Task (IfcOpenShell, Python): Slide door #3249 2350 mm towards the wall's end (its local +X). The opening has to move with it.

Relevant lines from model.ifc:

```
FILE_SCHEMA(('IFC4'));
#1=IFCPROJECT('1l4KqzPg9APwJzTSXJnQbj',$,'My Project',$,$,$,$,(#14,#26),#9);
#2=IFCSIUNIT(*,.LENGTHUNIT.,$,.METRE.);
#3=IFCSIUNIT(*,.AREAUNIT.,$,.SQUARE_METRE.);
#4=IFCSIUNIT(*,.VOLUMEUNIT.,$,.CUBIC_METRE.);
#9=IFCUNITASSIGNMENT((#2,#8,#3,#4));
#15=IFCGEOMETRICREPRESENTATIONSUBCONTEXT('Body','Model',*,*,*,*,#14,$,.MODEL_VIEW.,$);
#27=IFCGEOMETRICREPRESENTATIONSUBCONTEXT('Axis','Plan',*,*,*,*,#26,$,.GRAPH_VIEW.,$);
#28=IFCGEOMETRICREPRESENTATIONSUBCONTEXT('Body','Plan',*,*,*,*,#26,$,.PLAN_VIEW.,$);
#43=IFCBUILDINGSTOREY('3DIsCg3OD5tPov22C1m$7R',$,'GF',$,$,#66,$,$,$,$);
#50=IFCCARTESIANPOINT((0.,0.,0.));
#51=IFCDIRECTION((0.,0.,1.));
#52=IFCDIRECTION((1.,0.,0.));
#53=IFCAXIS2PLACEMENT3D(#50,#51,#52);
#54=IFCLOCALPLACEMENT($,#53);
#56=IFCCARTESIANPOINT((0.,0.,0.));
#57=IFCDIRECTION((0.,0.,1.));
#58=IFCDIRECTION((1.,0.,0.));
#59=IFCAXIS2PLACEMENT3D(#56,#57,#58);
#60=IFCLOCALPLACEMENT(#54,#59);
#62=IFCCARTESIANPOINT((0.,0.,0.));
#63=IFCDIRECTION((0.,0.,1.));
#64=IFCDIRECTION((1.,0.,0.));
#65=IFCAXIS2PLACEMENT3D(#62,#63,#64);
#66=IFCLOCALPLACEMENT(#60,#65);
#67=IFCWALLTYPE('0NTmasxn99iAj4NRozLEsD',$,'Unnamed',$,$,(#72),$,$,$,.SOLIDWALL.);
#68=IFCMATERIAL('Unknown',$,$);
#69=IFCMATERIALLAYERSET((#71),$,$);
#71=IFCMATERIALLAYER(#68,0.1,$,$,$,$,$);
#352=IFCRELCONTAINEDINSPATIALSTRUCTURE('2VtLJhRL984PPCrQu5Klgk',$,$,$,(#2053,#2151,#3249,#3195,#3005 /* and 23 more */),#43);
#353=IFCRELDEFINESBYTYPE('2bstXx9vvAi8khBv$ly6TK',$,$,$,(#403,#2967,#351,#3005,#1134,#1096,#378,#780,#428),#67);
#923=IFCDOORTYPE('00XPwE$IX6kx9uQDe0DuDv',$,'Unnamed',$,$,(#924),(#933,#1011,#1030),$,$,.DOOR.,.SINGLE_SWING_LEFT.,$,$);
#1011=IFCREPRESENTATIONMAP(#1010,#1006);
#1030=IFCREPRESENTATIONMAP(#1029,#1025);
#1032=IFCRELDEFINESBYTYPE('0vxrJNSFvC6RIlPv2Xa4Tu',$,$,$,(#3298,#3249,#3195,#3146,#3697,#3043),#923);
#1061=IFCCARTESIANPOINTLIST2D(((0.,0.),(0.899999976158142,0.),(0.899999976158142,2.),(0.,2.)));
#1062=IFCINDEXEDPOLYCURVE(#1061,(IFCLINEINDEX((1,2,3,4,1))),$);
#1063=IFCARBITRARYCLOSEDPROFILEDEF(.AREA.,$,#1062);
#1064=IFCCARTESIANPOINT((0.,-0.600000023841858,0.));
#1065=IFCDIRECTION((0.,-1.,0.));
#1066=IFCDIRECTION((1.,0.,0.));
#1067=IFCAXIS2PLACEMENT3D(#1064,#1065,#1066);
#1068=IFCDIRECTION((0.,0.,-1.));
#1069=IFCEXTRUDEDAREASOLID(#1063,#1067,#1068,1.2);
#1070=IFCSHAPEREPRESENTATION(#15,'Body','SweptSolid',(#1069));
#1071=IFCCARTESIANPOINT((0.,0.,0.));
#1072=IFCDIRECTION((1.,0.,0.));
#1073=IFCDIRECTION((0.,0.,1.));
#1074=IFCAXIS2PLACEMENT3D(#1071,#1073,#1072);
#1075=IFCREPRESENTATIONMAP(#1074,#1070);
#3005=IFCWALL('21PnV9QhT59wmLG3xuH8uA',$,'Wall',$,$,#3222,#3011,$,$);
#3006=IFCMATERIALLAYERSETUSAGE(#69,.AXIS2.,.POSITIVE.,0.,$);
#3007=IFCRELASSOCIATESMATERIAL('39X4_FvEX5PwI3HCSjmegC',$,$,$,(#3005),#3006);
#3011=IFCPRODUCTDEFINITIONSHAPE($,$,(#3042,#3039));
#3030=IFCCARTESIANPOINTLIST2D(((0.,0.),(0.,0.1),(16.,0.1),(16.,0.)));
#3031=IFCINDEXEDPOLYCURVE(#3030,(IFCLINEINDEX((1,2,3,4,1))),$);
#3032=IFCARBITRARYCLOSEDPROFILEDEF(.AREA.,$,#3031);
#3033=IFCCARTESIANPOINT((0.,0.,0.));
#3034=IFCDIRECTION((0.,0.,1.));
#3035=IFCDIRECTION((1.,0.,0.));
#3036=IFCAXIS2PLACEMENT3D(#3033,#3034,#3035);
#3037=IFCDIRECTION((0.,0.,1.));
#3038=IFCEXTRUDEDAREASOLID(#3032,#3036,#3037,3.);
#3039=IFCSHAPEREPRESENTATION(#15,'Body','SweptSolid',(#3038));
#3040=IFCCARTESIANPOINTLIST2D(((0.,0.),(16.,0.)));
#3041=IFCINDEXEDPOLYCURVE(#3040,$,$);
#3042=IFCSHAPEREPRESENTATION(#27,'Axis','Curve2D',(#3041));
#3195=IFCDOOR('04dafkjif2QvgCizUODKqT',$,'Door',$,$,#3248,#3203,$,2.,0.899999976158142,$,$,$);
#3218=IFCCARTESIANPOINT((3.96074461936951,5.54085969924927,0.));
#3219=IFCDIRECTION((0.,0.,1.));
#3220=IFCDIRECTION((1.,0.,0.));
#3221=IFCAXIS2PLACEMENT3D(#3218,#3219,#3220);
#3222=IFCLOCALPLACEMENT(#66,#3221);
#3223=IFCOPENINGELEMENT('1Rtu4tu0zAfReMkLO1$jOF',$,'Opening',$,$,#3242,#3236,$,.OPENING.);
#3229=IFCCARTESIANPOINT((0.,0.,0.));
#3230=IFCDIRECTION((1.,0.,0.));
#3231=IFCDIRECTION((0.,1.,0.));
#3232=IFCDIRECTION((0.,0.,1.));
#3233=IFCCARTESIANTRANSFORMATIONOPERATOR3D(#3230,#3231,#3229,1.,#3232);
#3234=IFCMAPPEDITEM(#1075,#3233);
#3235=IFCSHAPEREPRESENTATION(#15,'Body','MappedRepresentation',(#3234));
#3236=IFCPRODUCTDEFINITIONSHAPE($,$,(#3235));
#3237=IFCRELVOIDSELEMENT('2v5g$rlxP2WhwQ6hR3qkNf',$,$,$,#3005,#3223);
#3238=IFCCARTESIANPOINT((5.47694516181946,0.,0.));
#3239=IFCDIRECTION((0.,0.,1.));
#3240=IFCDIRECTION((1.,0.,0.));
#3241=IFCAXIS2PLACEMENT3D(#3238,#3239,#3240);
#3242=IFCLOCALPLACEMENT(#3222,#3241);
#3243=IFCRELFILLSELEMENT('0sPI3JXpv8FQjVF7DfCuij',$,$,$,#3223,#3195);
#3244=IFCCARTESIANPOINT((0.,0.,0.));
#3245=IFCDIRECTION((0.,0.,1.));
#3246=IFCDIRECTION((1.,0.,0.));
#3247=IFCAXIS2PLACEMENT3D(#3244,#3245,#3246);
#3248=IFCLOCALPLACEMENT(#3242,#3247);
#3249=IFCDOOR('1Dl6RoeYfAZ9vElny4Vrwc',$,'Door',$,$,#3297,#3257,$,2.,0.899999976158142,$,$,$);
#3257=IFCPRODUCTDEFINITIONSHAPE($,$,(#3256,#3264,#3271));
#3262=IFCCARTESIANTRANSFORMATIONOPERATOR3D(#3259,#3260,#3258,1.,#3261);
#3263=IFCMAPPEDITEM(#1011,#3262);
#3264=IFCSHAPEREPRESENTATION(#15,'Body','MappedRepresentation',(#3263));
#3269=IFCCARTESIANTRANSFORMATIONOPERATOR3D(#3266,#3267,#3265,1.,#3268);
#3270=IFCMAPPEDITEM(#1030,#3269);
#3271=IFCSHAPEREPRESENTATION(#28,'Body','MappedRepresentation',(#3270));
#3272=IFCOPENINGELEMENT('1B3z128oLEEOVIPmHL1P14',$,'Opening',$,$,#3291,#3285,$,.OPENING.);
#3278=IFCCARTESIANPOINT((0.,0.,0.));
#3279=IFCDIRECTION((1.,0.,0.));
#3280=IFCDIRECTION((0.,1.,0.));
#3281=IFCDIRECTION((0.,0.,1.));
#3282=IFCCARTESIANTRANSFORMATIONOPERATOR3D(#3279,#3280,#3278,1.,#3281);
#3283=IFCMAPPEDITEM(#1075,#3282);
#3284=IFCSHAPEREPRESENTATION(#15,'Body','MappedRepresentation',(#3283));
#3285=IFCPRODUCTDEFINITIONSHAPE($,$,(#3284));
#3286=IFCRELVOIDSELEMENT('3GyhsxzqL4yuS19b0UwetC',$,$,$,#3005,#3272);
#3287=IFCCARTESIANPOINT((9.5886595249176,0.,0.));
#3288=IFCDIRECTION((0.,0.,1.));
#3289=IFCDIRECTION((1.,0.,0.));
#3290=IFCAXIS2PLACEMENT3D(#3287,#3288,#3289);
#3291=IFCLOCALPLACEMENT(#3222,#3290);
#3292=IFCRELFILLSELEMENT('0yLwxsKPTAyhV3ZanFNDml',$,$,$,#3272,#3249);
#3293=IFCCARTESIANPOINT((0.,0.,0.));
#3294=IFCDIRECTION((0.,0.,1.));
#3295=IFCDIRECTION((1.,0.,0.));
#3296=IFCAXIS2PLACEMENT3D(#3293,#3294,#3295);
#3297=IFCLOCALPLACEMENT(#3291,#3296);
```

```python
import ifcopenshell
import ifcopenshell.api.geometry
import ifcopenshell.util.placement
import ifcopenshell.util.unit

model = ifcopenshell.open("model.ifc")
unit_scale = ifcopenshell.util.unit.calculate_unit_scale(model)

door = model.by_guid("1Dl6RoeYfAZ9vElny4Vrwc")
opening = door.FillsVoids[0].RelatingOpeningElement
wall = opening.VoidsElements[0].RelatingBuildingElement

wall_matrix = ifcopenshell.util.placement.get_local_placement(wall.ObjectPlacement)
shift = wall_matrix[:3, 0] * 2.35 / unit_scale
before = ifcopenshell.util.placement.get_local_placement(door.ObjectPlacement)[:3, 3].copy()

# The door is placed relative to its opening, so it follows when the opening moves.
matrix = ifcopenshell.util.placement.get_local_placement(opening.ObjectPlacement)
matrix[:3, 3] += shift
ifcopenshell.api.geometry.edit_object_placement(
    model, product=opening, matrix=matrix, is_si=False, should_transform_children=True
)

after = ifcopenshell.util.placement.get_local_placement(door.ObjectPlacement)[:3, 3]
print("door moved by", (after - before).round(3) + 0.0)

model.write("model_rev.ifc")
```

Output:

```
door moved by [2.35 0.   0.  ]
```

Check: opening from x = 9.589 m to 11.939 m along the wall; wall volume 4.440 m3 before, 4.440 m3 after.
